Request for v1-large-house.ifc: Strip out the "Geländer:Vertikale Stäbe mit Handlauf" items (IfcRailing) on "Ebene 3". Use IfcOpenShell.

First a look at what the model holds.

```python
import ifcopenshell
import ifcopenshell.util.element

model = ifcopenshell.open("v1-large-house.ifc")
print(model.schema)
storey = next(s for s in model.by_type("IfcBuildingStorey") if s.Name == "Ebene 3")
railings = [e for e in ifcopenshell.util.element.get_decomposition(storey) if e.is_a("IfcRailing")]
seen = {}
for e in railings:
    element_type = ifcopenshell.util.element.get_type(e)
    name = element_type.Name if element_type not in (None, e) else None
    seen[name] = seen.get(name, 0) + 1
for name, count in sorted(seen.items(), key=str):
    print(count, "x", name)
```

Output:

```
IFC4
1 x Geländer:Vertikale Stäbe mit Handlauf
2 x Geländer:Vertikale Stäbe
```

```python
import ifcopenshell
import ifcopenshell.api.root
import ifcopenshell.util.element

model = ifcopenshell.open("v1-large-house.ifc")

storey = next(s for s in model.by_type("IfcBuildingStorey") if s.Name == "Ebene 3")
railings = [e for e in ifcopenshell.util.element.get_decomposition(storey) if e.is_a("IfcRailing")]
targets = [e for e in railings if (t := ifcopenshell.util.element.get_type(e)) not in (None, e) and t.Name == "Geländer:Vertikale Stäbe mit Handlauf"]

for e in targets:
    ifcopenshell.api.root.remove_product(model, product=e)
print(len(targets), "removed")

model.write("v1-large-house-out.ifc")
```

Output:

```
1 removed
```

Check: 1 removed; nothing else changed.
